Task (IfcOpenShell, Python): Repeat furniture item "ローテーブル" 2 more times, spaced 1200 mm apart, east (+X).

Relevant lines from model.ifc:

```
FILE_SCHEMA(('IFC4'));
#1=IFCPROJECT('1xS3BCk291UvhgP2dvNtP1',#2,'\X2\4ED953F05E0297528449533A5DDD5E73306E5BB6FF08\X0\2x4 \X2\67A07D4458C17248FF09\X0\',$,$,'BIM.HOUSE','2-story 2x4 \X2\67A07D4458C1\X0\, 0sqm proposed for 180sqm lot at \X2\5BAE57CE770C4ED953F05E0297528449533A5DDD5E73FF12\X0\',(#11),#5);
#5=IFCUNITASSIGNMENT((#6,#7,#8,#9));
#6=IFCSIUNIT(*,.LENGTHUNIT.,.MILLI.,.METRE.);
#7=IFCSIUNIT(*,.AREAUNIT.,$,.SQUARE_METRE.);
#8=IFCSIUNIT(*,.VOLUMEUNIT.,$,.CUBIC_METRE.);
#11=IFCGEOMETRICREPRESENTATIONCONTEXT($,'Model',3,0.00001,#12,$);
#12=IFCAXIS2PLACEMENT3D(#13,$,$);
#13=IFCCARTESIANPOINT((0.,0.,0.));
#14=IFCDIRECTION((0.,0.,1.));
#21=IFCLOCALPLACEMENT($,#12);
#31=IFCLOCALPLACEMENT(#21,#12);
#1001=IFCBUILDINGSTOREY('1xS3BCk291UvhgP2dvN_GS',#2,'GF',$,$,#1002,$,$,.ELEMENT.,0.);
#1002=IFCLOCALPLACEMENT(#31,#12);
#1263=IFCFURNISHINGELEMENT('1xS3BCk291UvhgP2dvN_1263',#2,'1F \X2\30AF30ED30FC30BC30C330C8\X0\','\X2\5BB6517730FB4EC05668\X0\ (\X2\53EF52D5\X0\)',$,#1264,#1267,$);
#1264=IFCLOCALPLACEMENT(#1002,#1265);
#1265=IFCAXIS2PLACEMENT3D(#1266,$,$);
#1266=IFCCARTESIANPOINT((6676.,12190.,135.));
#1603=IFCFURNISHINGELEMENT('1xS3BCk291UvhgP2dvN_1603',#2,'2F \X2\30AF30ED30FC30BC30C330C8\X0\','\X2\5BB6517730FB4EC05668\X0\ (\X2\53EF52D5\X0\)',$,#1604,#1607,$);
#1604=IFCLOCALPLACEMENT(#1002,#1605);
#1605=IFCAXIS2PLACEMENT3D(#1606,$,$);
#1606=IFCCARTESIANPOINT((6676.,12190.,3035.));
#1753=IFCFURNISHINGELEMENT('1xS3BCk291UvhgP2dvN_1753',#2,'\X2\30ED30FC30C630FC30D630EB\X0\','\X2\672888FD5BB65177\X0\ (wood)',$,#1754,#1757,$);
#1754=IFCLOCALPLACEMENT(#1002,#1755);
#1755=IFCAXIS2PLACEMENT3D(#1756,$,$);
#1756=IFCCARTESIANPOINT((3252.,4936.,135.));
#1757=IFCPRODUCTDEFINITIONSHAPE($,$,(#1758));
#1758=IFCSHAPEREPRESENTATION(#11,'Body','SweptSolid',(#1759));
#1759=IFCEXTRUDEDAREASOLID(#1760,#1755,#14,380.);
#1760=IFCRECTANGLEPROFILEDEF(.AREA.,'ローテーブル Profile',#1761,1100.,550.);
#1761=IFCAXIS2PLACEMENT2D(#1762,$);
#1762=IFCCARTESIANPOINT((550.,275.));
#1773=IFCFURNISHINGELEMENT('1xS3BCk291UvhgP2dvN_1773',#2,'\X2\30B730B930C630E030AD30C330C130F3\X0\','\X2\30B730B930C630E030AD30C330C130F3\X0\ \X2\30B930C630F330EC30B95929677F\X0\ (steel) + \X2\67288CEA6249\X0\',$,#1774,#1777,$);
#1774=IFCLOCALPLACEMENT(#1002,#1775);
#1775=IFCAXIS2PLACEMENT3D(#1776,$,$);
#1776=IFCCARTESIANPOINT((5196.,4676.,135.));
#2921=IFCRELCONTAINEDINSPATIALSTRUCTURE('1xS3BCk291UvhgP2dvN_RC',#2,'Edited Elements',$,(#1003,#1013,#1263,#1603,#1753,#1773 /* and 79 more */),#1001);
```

```python
import numpy as np
import ifcopenshell
import ifcopenshell.api.geometry
import ifcopenshell.api.root
import ifcopenshell.util.element
import ifcopenshell.util.placement
import ifcopenshell.util.unit

model = ifcopenshell.open("model.ifc")
unit_scale = ifcopenshell.util.unit.calculate_unit_scale(model)


def reuse_history(source, copy):
    """copy_class also copies each property set's owner history, people and application; keep the originals."""
    for rel in copy.IsDefinedBy:
        if rel.is_a("IfcRelDefinesByProperties") and (history := rel.RelatingPropertyDefinition.OwnerHistory):
            rel.RelatingPropertyDefinition.OwnerHistory = source.OwnerHistory
            ifcopenshell.util.element.remove_deep2(model, history)


source = model.by_guid("1xS3BCk291UvhgP2dvN_1753")
base = ifcopenshell.util.placement.get_local_placement(source.ObjectPlacement)
step = np.array([1.0, 0.0, 0.0]) * 1.2 / unit_scale

for i in range(1, 3):
    copy = ifcopenshell.api.root.copy_class(model, product=source)
    copy.Representation = ifcopenshell.util.element.copy_deep(
        model, source.Representation, exclude=["IfcGeometricRepresentationContext", "IfcRepresentationMap"]
    )
    reuse_history(source, copy)
    matrix = base.copy()
    matrix[:3, 3] += i * step
    print("added at", matrix[:3, 3].round(3) + 0.0)
    ifcopenshell.api.geometry.edit_object_placement(model, product=copy, matrix=matrix, is_si=False)

model.write("model-out.ifc")
```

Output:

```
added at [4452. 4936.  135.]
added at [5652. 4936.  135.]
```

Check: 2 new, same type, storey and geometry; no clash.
